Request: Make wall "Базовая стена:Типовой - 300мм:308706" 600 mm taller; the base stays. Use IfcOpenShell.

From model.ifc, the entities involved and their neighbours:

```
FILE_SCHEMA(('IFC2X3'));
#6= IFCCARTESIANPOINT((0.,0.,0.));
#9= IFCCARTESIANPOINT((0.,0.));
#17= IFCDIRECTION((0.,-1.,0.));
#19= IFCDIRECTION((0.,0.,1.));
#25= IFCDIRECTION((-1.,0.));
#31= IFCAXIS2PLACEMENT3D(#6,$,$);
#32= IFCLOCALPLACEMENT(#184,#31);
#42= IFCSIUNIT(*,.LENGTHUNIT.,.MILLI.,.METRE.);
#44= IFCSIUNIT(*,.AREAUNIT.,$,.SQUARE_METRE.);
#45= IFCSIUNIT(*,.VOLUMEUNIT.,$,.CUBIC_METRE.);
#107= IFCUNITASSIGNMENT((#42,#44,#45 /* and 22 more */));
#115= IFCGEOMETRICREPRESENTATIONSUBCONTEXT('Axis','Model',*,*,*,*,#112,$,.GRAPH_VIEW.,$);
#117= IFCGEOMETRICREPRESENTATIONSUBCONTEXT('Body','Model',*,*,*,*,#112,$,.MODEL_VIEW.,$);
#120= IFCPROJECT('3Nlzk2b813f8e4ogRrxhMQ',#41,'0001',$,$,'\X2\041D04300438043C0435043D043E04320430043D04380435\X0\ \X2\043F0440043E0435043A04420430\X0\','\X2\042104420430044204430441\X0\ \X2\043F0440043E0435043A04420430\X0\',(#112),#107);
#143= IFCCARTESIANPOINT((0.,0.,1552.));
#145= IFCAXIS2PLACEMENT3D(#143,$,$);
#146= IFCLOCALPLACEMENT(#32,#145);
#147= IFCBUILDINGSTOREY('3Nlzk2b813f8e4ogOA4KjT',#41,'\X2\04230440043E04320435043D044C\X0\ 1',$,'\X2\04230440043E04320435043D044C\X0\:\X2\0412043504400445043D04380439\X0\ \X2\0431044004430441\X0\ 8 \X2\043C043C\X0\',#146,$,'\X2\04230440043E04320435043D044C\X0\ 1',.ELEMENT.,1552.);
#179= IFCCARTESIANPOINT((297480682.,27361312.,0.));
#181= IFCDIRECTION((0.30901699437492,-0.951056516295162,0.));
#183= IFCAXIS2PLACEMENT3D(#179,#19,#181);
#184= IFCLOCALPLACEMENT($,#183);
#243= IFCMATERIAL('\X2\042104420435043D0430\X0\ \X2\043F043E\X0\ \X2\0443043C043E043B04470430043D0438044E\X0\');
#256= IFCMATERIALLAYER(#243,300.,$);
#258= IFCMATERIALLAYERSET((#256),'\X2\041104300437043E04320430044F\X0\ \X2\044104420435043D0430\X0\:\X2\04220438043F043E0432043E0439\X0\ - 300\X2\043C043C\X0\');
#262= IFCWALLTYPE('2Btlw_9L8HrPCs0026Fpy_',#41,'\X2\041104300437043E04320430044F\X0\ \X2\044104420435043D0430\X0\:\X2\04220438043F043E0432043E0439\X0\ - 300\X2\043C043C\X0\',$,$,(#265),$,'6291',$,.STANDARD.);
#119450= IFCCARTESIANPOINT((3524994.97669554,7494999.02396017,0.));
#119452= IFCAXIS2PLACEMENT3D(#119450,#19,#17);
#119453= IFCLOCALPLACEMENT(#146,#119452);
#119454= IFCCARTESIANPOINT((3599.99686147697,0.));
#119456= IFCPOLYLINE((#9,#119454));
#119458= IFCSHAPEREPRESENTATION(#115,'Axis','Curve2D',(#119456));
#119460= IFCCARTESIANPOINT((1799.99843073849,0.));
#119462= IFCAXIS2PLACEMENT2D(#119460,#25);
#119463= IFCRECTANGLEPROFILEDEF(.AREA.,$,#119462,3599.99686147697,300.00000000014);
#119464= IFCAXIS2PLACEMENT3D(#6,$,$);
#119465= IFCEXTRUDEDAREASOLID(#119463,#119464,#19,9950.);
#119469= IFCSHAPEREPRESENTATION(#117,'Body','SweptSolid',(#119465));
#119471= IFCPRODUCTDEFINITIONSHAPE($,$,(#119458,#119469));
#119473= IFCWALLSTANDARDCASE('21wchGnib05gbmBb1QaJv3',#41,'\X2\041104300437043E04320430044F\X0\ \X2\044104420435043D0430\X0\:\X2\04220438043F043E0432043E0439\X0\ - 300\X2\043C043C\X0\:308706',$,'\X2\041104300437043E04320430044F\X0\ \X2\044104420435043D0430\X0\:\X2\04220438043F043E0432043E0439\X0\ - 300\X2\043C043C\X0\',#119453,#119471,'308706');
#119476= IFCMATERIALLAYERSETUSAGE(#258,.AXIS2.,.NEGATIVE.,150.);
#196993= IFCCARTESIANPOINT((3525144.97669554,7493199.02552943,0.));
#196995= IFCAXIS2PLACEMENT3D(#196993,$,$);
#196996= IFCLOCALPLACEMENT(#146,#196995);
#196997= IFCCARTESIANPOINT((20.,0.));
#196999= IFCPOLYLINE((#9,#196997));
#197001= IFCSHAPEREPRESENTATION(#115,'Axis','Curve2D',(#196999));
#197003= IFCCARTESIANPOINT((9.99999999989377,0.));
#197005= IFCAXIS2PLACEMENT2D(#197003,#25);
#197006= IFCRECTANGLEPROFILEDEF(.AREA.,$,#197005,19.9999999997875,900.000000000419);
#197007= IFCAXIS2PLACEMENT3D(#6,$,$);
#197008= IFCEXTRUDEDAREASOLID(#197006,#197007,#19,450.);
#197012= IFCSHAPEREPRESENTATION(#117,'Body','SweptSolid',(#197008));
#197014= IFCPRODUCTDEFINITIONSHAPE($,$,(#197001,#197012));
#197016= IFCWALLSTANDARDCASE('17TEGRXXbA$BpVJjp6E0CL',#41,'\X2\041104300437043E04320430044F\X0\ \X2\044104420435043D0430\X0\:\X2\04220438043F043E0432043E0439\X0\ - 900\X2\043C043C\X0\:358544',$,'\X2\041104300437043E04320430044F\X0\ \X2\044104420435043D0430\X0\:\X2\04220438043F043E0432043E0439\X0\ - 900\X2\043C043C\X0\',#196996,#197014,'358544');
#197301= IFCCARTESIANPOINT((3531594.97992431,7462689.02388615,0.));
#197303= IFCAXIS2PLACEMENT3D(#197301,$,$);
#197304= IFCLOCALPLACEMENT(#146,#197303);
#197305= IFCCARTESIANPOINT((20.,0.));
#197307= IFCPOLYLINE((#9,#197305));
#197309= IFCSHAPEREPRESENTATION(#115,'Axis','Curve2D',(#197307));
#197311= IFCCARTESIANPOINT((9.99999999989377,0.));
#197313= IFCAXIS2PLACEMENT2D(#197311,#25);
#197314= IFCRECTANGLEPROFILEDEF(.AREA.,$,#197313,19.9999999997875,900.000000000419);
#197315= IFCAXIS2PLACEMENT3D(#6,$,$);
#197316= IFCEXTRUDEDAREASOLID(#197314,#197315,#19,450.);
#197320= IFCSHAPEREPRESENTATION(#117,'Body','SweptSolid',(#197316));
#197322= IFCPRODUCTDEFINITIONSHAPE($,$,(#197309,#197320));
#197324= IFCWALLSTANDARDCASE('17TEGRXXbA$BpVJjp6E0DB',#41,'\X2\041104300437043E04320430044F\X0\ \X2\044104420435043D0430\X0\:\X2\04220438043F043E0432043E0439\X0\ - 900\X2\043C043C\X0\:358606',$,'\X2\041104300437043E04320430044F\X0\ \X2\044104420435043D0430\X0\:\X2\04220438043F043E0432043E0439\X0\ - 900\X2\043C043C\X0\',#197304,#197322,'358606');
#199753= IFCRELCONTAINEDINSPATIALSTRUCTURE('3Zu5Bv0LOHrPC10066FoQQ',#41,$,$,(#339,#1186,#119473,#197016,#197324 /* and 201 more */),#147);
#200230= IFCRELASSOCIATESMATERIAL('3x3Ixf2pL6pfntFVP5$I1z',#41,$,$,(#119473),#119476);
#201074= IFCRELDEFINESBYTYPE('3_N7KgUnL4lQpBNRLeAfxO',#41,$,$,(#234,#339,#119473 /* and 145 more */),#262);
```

```python
import ifcopenshell
import ifcopenshell.geom
import ifcopenshell.util.representation
import ifcopenshell.util.shape
import ifcopenshell.util.unit

model = ifcopenshell.open("model.ifc")
unit_scale = ifcopenshell.util.unit.calculate_unit_scale(model)
settings = ifcopenshell.geom.settings()


def volume(element):
    """Net volume in cubic metres, openings subtracted."""
    shape = ifcopenshell.geom.create_shape(settings, element)
    return ifcopenshell.util.shape.get_volume(shape.geometry)


wall = model.by_guid("21wchGnib05gbmBb1QaJv3")
before = volume(wall)

body = ifcopenshell.util.representation.get_representation(wall, "Model", "Body")
solid = body.Items[0]
old_height = solid.Depth
solid.Depth += 0.6 / unit_scale
after = volume(wall)

print(f"height {old_height:g} -> {solid.Depth:g}, volume {before:.3f} -> {after:.3f} m3")

model.write("model_updated.ifc")
```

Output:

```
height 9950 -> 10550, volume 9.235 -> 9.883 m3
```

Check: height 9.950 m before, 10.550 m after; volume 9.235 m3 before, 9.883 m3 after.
